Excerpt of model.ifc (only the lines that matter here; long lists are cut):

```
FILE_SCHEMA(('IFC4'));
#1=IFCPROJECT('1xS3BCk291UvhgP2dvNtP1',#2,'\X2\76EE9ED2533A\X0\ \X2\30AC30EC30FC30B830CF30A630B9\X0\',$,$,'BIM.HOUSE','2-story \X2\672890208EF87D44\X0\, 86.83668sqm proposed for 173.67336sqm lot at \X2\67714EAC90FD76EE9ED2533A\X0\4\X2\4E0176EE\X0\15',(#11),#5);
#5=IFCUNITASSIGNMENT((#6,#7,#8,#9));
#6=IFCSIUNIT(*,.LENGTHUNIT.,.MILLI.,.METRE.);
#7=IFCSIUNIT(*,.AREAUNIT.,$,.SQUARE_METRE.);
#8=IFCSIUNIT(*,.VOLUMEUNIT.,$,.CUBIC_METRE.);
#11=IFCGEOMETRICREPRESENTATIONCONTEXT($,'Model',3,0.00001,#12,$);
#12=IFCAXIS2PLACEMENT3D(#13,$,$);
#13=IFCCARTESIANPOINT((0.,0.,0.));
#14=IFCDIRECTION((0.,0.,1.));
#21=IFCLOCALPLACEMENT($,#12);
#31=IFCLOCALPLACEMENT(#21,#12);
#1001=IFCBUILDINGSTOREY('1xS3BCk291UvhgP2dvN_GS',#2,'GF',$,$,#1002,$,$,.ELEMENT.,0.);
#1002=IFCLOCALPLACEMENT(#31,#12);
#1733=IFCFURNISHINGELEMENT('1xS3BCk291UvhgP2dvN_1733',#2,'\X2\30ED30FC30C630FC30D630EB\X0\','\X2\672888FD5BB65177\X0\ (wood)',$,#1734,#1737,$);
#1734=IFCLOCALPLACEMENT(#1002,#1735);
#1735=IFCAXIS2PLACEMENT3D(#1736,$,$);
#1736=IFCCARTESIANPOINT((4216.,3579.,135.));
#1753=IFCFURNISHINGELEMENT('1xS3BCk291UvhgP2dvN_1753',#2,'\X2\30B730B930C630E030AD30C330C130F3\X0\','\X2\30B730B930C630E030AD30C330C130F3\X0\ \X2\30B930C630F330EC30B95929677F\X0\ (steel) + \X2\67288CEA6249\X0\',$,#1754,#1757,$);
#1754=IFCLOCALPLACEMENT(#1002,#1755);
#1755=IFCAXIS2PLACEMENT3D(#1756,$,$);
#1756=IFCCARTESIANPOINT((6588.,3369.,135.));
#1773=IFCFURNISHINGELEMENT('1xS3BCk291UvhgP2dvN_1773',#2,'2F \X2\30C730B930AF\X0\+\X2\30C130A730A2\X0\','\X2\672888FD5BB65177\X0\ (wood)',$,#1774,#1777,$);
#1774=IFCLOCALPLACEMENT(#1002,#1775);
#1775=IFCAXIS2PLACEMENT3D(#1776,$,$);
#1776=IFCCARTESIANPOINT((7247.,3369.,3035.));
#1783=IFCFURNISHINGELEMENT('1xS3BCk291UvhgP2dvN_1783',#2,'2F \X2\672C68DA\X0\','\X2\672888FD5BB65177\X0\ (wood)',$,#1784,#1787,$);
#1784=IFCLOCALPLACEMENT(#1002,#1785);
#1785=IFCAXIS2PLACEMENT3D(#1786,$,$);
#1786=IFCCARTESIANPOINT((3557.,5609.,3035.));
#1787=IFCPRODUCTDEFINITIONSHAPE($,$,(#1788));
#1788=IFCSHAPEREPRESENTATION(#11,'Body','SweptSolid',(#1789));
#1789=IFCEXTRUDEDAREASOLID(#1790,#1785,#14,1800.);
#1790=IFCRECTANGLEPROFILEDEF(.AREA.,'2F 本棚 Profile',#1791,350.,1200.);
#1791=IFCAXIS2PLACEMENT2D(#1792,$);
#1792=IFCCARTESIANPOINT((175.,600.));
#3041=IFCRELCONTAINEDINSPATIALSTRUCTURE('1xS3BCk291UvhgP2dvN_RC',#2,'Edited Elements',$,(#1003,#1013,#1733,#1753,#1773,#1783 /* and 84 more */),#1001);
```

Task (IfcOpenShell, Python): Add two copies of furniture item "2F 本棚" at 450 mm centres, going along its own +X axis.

```python
import ifcopenshell
import ifcopenshell.api.geometry
import ifcopenshell.api.root
import ifcopenshell.util.element
import ifcopenshell.util.placement

model = ifcopenshell.open("model.ifc")


def reuse_history(source, copy):
    """copy_class also copies each property set's owner history, people and application; keep the originals."""
    for rel in copy.IsDefinedBy:
        if rel.is_a("IfcRelDefinesByProperties") and (history := rel.RelatingPropertyDefinition.OwnerHistory):
            rel.RelatingPropertyDefinition.OwnerHistory = source.OwnerHistory
            ifcopenshell.util.element.remove_deep2(model, history)


source = model.by_guid("1xS3BCk291UvhgP2dvN_1783")
base = ifcopenshell.util.placement.get_local_placement(source.ObjectPlacement)
step = base[:3, 0] * 450.0

for i in range(1, 3):
    copy = ifcopenshell.api.root.copy_class(model, product=source)
    copy.Representation = ifcopenshell.util.element.copy_deep(
        model, source.Representation, exclude=["IfcGeometricRepresentationContext", "IfcRepresentationMap"]
    )
    reuse_history(source, copy)
    matrix = base.copy()
    matrix[:3, 3] += i * step
    print("added at", matrix[:3, 3].round(3) + 0.0)
    ifcopenshell.api.geometry.edit_object_placement(model, product=copy, matrix=matrix, is_si=False)

model.write("model_v2.ifc")
```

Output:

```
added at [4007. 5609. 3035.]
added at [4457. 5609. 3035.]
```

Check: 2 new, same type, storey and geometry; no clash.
